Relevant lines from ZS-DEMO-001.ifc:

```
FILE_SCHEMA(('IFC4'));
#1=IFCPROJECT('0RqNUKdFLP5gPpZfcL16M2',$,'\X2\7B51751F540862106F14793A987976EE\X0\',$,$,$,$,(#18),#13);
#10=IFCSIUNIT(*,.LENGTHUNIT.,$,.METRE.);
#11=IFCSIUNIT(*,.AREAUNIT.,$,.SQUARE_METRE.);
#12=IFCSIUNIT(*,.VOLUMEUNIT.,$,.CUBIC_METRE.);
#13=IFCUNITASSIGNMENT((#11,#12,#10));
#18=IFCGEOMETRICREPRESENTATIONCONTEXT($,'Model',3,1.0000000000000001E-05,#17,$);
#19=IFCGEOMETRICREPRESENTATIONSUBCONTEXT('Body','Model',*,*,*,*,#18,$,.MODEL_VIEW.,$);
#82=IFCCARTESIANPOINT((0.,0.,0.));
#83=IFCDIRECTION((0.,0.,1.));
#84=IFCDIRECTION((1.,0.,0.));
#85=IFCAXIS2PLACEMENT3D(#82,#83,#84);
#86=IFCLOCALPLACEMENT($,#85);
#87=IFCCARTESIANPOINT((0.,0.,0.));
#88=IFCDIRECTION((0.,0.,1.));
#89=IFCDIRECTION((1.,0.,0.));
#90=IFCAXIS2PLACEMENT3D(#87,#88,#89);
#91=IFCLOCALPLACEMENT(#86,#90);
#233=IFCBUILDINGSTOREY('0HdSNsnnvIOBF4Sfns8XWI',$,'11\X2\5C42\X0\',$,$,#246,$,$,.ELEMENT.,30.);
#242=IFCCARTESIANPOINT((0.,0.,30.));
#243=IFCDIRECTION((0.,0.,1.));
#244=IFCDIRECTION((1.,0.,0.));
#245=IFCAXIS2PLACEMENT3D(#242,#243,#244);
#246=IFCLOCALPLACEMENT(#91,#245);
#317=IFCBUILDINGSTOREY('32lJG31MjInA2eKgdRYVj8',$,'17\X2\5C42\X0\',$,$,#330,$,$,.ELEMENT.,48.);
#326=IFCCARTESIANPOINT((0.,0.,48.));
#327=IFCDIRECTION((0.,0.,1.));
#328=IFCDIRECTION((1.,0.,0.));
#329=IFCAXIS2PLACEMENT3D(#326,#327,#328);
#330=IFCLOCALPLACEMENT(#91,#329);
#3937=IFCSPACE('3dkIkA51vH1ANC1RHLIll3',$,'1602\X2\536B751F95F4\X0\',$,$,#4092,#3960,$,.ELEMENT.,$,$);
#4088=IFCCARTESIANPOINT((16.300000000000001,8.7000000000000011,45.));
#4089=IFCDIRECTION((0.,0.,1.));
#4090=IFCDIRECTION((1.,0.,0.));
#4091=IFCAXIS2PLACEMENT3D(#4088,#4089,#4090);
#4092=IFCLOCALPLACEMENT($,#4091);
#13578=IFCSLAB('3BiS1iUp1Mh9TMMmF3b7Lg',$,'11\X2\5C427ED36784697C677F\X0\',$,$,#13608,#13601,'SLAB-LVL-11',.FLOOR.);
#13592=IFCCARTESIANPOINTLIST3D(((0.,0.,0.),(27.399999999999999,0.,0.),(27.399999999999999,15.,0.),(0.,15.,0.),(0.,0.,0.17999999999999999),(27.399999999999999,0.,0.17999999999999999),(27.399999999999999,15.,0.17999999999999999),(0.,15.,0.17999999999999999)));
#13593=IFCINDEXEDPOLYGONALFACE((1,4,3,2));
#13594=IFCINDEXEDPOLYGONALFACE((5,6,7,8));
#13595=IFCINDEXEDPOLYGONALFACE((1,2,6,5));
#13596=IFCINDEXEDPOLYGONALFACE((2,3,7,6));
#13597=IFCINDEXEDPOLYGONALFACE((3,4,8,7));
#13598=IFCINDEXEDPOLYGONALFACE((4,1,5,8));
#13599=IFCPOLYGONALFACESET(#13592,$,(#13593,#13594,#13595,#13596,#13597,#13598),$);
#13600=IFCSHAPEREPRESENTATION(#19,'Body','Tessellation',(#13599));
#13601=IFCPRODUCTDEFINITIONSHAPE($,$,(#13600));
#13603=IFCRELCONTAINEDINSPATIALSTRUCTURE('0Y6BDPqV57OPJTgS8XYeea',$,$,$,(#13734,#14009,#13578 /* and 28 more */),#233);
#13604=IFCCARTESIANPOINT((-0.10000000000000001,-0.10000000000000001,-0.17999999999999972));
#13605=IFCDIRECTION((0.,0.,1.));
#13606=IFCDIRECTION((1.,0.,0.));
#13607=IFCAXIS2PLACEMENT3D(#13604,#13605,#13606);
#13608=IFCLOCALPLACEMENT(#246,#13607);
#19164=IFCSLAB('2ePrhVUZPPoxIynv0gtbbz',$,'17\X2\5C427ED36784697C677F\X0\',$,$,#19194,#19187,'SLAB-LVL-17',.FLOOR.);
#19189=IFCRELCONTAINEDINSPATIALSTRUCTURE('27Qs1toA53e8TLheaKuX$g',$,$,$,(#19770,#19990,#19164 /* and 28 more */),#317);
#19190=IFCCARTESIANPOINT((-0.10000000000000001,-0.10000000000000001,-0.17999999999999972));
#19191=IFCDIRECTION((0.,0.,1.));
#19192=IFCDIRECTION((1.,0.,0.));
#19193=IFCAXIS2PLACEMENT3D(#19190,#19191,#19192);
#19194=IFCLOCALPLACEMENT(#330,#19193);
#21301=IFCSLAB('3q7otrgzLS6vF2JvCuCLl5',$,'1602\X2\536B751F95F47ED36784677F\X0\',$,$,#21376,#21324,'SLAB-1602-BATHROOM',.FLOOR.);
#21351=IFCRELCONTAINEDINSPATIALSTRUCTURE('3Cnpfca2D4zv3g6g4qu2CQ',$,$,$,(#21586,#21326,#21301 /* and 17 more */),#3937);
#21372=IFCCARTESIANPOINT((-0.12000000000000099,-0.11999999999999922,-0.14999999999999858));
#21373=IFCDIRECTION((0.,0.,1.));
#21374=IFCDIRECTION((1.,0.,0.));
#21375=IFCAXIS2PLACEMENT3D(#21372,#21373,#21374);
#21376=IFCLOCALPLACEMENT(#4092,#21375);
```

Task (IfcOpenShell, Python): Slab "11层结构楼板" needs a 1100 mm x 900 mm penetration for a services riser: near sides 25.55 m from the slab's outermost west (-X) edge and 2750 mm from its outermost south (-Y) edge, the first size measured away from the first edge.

```python
import numpy as np
import ifcopenshell
import ifcopenshell.api.feature
import ifcopenshell.api.geometry
import ifcopenshell.api.root
import ifcopenshell.geom
import ifcopenshell.util.placement
import ifcopenshell.util.representation
import ifcopenshell.util.shape
import ifcopenshell.util.unit

model = ifcopenshell.open("ZS-DEMO-001.ifc")
unit_scale = ifcopenshell.util.unit.calculate_unit_scale(model)
settings = ifcopenshell.geom.settings()


def volume(element):
    """Net volume in cubic metres, openings subtracted."""
    shape = ifcopenshell.geom.create_shape(settings, element)
    return ifcopenshell.util.shape.get_volume(shape.geometry)


slab = model.by_guid("3BiS1iUp1Mh9TMMmF3b7Lg")
before = volume(slab)

# Extent in the slab's own axes, in metres. The edges named are its -X and -Y sides.
slab_shape = ifcopenshell.geom.create_shape(settings, slab)
vertices = ifcopenshell.util.shape.get_vertices(slab_shape.geometry)
x_min, y_min, bottom = vertices.min(axis=0)
top = vertices[:, 2].max()

opening = ifcopenshell.api.root.create_entity(model, ifc_class="IfcOpeningElement", name="Services riser opening", predefined_type="OPENING")
context = ifcopenshell.util.representation.get_context(model, "Model", "Body", "MODEL_VIEW")
width, depth = 1.1, 0.9
outline = [(0.0, 0.0), (width, 0.0), (width, depth), (0.0, depth), (0.0, 0.0)]
# Overshoot both faces by 50 mm so the cut is clean.
shape = ifcopenshell.api.geometry.add_slab_representation(
    model, context=context, depth=top - bottom + 0.1, polyline=outline
)
ifcopenshell.api.geometry.assign_representation(model, product=opening, representation=shape)

matrix = ifcopenshell.util.placement.get_local_placement(slab.ObjectPlacement)
matrix[:, 3] = matrix @ np.append(np.array([x_min + 25.55, y_min + 2.75, bottom - 0.05]) / unit_scale, 1.0)
ifcopenshell.api.geometry.edit_object_placement(model, product=opening, matrix=matrix, is_si=False)
ifcopenshell.api.feature.add_feature(model, feature=opening, element=slab)

after = volume(slab)

print(f"slab volume {before:.3f} -> {after:.3f} m3")

model.write("ZS-DEMO-001_v2.ifc")
```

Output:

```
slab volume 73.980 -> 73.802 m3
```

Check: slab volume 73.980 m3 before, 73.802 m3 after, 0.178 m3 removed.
